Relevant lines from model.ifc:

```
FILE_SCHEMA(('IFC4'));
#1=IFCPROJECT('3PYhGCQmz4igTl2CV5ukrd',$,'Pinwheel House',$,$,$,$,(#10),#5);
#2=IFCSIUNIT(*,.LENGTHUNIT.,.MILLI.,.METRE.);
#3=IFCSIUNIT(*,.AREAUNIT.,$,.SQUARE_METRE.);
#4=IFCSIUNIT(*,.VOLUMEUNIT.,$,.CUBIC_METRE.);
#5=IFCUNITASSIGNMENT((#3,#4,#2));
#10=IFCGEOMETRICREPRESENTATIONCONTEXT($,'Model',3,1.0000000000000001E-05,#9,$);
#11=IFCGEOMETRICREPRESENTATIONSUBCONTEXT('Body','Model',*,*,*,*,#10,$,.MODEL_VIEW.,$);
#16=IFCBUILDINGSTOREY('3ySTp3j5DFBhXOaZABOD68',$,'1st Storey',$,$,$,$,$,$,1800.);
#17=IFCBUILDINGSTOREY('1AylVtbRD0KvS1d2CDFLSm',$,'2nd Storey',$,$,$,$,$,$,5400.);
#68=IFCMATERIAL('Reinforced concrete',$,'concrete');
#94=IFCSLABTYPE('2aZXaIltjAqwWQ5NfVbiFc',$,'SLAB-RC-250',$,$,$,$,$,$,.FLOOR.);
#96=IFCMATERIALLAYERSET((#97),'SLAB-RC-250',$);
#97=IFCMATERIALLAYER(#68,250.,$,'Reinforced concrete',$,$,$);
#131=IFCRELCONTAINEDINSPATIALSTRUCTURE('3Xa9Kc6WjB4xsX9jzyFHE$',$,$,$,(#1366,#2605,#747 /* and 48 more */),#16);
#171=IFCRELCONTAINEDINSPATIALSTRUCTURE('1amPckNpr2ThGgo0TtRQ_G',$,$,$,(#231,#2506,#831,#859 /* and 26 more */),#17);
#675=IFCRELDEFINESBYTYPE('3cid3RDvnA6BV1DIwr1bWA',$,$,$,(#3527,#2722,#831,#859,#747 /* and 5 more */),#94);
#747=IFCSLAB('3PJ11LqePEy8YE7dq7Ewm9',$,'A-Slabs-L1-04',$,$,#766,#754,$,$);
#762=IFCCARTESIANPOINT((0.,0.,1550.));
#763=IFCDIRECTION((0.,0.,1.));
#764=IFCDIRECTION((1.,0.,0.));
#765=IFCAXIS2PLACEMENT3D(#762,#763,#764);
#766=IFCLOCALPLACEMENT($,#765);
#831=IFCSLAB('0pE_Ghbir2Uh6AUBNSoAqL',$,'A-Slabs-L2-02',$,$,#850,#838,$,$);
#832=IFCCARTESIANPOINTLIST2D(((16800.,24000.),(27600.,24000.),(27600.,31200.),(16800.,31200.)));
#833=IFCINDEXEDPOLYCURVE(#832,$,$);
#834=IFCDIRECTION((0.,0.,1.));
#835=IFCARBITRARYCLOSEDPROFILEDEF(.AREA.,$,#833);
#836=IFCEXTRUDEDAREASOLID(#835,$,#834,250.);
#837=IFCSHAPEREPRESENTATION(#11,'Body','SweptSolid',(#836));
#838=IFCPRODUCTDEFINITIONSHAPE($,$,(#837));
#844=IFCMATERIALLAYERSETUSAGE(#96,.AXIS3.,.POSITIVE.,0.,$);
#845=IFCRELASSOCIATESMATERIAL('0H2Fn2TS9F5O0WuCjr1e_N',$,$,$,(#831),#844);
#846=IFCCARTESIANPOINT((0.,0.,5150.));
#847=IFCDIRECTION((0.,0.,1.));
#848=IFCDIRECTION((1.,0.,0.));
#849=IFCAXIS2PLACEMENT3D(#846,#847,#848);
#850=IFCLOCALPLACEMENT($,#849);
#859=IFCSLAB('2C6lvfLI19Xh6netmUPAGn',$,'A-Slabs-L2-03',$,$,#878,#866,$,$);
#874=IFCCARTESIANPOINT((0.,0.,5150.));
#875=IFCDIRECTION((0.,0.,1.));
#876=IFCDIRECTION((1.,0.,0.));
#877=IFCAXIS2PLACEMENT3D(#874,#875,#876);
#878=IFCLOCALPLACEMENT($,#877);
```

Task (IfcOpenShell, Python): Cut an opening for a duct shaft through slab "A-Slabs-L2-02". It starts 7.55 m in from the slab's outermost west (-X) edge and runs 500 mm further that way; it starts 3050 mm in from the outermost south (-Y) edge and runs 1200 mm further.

```python
import numpy as np
import ifcopenshell
import ifcopenshell.api.feature
import ifcopenshell.api.geometry
import ifcopenshell.api.root
import ifcopenshell.geom
import ifcopenshell.util.placement
import ifcopenshell.util.representation
import ifcopenshell.util.shape
import ifcopenshell.util.unit

model = ifcopenshell.open("model.ifc")
unit_scale = ifcopenshell.util.unit.calculate_unit_scale(model)
settings = ifcopenshell.geom.settings()


def volume(element):
    """Net volume in cubic metres, openings subtracted."""
    shape = ifcopenshell.geom.create_shape(settings, element)
    return ifcopenshell.util.shape.get_volume(shape.geometry)


slab = model.by_guid("0pE_Ghbir2Uh6AUBNSoAqL")
before = volume(slab)

# Extent in the slab's own axes, in metres. The edges named are its -X and -Y sides.
slab_shape = ifcopenshell.geom.create_shape(settings, slab)
vertices = ifcopenshell.util.shape.get_vertices(slab_shape.geometry)
x_min, y_min, bottom = vertices.min(axis=0)
top = vertices[:, 2].max()

opening = ifcopenshell.api.root.create_entity(model, ifc_class="IfcOpeningElement", name="Duct shaft opening", predefined_type="OPENING")
context = ifcopenshell.util.representation.get_context(model, "Model", "Body", "MODEL_VIEW")
width, depth = 0.5, 1.2
outline = [(0.0, 0.0), (width, 0.0), (width, depth), (0.0, depth), (0.0, 0.0)]
# Overshoot both faces by 50 mm so the cut is clean.
shape = ifcopenshell.api.geometry.add_slab_representation(
    model, context=context, depth=top - bottom + 0.1, polyline=outline
)
ifcopenshell.api.geometry.assign_representation(model, product=opening, representation=shape)

matrix = ifcopenshell.util.placement.get_local_placement(slab.ObjectPlacement)
matrix[:, 3] = matrix @ np.append(np.array([x_min + 7.55, y_min + 3.05, bottom - 0.05]) / unit_scale, 1.0)
ifcopenshell.api.geometry.edit_object_placement(model, product=opening, matrix=matrix, is_si=False)
ifcopenshell.api.feature.add_feature(model, feature=opening, element=slab)

after = volume(slab)

print(f"slab volume {before:.3f} -> {after:.3f} m3")

model.write("model_edited.ifc")
```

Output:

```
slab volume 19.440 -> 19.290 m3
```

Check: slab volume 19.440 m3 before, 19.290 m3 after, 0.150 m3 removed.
